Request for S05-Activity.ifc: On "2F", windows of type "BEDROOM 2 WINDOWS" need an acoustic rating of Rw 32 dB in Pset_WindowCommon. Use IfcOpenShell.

First a look at what the model holds.

```python
import ifcopenshell
import ifcopenshell.util.element

model = ifcopenshell.open("S05-Activity.ifc")
print(model.schema)
storey = next(s for s in model.by_type("IfcBuildingStorey") if s.Name == "2F")
windows = [e for e in ifcopenshell.util.element.get_decomposition(storey) if e.is_a("IfcWindow")]
seen = {}
for e in windows:
    element_type = ifcopenshell.util.element.get_type(e)
    key = (element_type.Name if element_type != e and element_type else None, ifcopenshell.util.element.get_pset(e, "Pset_WindowCommon", "AcousticRating"))
    seen[key] = seen.get(key, 0) + 1
for (name, value), count in sorted(seen.items(), key=str):
    print(count, "x", name, "|", value)
```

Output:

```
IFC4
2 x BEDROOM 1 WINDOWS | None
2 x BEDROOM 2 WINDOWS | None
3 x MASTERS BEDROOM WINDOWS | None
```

```python
import ifcopenshell
import ifcopenshell.api.pset
import ifcopenshell.util.element

model = ifcopenshell.open("S05-Activity.ifc")

storey = next(s for s in model.by_type("IfcBuildingStorey") if s.Name == "2F")
windows = [e for e in ifcopenshell.util.element.get_decomposition(storey) if e.is_a("IfcWindow")]

count = 0
for e in windows:
    element_type = ifcopenshell.util.element.get_type(e)
    if element_type in (None, e) or element_type.Name != "BEDROOM 2 WINDOWS":
        continue
    # add_pset returns the element's existing set when there is one.
    pset = ifcopenshell.api.pset.add_pset(model, product=e, name="Pset_WindowCommon")
    ifcopenshell.api.pset.edit_pset(model, pset=pset, properties={"AcousticRating": "Rw 32 dB"})
    count += 1

print(count, "windows updated")

model.write("S05-Activity_updated.ifc")
```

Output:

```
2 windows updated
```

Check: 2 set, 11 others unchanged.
